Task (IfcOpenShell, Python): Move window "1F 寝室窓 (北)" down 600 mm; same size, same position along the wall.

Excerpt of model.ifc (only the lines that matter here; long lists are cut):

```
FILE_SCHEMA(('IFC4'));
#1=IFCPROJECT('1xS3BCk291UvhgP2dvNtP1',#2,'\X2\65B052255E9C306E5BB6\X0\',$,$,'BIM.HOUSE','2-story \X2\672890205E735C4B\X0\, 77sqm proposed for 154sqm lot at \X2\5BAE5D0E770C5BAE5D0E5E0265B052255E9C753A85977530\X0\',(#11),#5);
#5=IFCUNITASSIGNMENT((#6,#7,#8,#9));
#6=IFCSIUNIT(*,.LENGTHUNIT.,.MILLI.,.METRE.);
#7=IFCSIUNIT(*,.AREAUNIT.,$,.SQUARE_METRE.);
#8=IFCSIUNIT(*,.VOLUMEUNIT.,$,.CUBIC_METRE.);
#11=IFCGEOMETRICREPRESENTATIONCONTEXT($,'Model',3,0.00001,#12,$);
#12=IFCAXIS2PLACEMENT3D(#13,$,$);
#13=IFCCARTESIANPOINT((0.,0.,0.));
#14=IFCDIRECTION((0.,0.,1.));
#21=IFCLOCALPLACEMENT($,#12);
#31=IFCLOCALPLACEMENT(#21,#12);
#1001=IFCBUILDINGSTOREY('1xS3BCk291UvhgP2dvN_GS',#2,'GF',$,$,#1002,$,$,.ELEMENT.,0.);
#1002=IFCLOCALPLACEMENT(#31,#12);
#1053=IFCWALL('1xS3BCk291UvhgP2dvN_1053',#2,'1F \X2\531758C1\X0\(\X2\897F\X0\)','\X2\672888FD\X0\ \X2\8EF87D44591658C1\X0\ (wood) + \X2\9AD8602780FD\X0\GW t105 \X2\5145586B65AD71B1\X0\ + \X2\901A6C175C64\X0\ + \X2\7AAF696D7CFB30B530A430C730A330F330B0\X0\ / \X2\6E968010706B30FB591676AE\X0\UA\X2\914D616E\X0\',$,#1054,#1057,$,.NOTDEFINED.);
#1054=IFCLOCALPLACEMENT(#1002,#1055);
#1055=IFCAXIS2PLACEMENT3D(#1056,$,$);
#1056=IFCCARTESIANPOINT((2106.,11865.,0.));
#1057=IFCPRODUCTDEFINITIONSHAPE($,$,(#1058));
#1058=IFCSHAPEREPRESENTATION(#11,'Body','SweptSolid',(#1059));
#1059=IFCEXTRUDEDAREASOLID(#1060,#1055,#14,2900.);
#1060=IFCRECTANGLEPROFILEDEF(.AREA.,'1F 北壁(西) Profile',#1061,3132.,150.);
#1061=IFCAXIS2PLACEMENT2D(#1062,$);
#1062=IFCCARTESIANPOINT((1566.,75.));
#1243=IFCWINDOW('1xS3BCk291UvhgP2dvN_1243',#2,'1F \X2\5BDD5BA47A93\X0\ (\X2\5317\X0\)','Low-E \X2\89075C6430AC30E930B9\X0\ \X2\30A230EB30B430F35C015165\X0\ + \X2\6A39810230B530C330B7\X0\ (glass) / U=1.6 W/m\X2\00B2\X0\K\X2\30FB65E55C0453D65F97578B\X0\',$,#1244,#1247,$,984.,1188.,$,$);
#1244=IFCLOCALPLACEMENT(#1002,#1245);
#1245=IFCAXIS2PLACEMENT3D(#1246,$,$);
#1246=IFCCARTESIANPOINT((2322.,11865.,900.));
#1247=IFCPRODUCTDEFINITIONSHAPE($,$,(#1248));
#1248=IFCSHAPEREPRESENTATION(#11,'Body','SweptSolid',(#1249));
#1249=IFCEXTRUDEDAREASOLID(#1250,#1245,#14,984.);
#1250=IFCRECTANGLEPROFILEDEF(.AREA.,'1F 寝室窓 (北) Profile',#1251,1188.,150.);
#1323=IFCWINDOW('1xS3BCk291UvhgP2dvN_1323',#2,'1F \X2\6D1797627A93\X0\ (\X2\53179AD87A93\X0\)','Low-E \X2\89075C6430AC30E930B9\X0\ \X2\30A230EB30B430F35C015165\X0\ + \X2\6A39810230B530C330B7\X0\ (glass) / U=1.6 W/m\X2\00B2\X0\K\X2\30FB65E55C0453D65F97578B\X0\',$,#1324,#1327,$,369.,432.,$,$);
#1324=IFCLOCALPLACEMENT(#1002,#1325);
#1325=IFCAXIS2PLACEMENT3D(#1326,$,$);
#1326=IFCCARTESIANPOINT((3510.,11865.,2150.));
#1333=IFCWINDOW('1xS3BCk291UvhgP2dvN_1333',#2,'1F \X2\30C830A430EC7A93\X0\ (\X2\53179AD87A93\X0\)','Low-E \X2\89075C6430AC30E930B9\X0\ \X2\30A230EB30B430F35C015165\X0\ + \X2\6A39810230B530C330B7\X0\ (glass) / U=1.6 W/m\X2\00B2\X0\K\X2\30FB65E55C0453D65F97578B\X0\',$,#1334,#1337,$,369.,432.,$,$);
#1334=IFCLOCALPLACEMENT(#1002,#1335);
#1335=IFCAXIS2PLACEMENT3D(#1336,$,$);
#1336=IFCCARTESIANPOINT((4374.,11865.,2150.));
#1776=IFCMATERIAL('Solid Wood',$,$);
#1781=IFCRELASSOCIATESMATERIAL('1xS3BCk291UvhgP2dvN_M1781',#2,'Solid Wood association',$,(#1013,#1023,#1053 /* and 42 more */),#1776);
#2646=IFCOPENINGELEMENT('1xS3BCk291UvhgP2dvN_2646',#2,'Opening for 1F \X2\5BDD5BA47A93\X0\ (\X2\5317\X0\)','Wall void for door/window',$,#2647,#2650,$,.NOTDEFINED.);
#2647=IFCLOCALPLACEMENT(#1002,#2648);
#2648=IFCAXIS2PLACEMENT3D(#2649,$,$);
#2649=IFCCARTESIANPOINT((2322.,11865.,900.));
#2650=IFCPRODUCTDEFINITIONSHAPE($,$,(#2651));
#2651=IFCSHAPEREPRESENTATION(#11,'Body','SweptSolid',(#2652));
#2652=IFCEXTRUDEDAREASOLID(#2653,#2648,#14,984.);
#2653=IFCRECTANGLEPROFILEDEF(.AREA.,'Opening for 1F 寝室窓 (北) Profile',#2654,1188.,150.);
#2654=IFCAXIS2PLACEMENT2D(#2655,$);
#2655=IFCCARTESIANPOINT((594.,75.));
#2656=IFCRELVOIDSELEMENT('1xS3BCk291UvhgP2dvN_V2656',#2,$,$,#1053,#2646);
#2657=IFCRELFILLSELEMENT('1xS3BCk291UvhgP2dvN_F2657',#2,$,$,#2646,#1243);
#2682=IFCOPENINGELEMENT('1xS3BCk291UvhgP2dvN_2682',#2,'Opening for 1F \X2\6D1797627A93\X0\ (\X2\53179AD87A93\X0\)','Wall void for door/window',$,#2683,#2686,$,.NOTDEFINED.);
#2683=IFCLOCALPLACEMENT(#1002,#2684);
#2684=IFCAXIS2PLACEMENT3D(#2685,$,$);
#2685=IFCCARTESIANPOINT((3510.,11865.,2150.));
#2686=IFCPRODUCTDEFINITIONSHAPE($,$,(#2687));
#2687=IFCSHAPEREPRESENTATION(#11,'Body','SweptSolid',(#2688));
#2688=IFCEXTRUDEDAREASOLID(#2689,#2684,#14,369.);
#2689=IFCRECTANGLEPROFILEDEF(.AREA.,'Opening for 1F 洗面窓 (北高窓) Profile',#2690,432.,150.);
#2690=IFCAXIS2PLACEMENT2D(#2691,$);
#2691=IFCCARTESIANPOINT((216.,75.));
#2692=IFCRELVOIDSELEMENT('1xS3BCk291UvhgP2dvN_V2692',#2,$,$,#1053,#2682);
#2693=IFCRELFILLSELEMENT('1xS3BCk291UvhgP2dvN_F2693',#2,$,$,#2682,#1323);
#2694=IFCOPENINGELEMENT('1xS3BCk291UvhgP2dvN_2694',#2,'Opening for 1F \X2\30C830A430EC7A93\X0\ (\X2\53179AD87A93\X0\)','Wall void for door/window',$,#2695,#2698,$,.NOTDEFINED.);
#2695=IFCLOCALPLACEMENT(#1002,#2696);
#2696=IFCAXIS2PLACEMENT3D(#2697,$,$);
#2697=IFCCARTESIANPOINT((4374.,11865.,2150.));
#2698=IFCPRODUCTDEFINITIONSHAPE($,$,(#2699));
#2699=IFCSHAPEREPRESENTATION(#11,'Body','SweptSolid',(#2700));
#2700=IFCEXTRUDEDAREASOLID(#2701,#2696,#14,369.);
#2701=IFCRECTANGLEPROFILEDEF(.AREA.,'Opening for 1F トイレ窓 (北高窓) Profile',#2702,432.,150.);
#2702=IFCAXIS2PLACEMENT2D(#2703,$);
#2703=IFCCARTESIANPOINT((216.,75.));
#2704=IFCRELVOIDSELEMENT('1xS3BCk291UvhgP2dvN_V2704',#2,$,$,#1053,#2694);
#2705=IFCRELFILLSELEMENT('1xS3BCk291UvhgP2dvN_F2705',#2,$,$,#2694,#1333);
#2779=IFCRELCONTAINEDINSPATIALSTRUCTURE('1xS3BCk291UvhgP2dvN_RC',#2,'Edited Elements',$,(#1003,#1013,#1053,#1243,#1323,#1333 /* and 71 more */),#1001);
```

```python
import numpy as np
import ifcopenshell
import ifcopenshell.api.geometry
import ifcopenshell.util.placement
import ifcopenshell.util.unit

model = ifcopenshell.open("model.ifc")
unit_scale = ifcopenshell.util.unit.calculate_unit_scale(model)

window = model.by_guid("1xS3BCk291UvhgP2dvN_1243")
opening = window.FillsVoids[0].RelatingOpeningElement
dz = -0.6 / unit_scale

shift = np.array([0.0, 0.0, dz])
# The window is not placed relative to its opening, so move both.
for product in (opening, window):
    matrix = ifcopenshell.util.placement.get_local_placement(product.ObjectPlacement)
    matrix[:3, 3] += shift
    ifcopenshell.api.geometry.edit_object_placement(model, product=product, matrix=matrix, is_si=False)

print(f"moved by {dz * unit_scale:+.3f} m")

model.write("model_v2.ifc")
```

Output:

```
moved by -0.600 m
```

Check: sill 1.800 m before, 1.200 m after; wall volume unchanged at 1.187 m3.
